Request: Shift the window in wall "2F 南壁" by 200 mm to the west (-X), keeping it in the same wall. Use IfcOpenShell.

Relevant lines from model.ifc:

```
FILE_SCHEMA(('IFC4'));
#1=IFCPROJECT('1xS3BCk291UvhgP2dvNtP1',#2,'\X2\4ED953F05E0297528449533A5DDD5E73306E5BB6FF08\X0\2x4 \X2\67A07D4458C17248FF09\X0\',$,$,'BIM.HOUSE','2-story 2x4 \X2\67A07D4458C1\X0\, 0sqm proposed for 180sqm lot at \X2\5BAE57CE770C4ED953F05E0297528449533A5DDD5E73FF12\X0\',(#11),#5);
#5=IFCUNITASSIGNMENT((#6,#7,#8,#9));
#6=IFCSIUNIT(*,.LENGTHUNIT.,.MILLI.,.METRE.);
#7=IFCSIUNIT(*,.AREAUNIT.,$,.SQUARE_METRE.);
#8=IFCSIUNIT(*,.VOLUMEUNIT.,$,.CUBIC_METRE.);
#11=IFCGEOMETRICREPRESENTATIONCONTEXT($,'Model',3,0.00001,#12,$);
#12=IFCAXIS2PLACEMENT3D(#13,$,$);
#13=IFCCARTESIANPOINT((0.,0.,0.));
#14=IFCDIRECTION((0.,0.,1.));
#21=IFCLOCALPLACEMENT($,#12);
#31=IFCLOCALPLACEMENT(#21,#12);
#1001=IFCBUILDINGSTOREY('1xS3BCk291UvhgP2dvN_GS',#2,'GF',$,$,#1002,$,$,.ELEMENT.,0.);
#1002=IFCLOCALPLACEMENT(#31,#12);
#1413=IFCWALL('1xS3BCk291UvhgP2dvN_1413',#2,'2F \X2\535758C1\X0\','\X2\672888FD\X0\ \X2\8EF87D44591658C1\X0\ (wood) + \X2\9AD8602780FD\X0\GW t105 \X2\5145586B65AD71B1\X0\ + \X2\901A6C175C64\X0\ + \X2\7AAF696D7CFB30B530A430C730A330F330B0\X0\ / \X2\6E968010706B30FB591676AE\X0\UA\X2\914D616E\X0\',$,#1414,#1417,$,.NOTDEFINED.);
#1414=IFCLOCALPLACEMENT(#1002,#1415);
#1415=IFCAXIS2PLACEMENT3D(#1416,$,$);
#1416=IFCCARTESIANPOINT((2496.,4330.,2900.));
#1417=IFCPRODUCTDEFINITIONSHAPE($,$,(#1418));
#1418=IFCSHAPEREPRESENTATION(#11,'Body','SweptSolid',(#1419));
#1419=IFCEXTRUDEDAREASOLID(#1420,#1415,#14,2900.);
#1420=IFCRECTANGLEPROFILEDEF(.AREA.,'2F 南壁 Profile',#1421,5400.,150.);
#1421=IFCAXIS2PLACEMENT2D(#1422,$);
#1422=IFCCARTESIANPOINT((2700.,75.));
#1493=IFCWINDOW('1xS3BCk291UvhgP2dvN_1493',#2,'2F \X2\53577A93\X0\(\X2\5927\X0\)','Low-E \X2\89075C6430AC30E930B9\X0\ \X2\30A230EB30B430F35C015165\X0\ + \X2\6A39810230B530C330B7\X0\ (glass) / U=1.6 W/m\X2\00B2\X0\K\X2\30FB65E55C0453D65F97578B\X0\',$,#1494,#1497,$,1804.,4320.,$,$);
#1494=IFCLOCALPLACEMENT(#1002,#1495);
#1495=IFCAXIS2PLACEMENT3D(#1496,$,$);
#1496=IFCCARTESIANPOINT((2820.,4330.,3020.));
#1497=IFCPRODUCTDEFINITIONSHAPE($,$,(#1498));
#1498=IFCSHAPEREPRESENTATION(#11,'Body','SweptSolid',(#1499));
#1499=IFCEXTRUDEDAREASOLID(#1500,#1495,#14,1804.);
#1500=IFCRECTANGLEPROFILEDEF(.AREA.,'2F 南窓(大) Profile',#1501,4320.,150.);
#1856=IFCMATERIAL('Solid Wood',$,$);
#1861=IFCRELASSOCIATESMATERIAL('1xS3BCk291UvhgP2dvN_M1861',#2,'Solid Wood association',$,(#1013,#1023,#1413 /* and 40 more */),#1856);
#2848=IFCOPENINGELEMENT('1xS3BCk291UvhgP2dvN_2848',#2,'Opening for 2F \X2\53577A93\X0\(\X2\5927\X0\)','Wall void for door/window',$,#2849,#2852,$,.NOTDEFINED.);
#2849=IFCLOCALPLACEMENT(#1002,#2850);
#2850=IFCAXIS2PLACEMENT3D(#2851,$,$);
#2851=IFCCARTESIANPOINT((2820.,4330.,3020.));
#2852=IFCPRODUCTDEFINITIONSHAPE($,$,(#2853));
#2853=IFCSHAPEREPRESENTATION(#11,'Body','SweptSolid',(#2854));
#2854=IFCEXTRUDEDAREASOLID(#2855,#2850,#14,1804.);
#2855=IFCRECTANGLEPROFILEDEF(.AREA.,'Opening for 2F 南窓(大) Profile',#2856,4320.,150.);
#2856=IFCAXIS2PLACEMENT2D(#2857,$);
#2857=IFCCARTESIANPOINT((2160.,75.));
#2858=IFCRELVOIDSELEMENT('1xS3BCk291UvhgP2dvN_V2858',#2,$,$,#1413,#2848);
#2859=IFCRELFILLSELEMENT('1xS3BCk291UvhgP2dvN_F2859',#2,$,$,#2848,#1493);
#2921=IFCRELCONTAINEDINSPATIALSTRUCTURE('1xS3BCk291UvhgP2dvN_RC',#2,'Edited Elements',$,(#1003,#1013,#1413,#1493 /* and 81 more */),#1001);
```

```python
import ifcopenshell
import ifcopenshell.api.geometry
import ifcopenshell.util.placement

model = ifcopenshell.open("model.ifc")

window = model.by_id(1493)
opening = window.FillsVoids[0].RelatingOpeningElement
wall = opening.VoidsElements[0].RelatingBuildingElement

wall_matrix = ifcopenshell.util.placement.get_local_placement(wall.ObjectPlacement)
shift = wall_matrix[:3, 0] * -200.0
before = ifcopenshell.util.placement.get_local_placement(window.ObjectPlacement)[:3, 3].copy()

# The window is not placed relative to its opening, so move both.
for product in (opening, window):
    matrix = ifcopenshell.util.placement.get_local_placement(product.ObjectPlacement)
    matrix[:3, 3] += shift
    ifcopenshell.api.geometry.edit_object_placement(model, product=product, matrix=matrix, is_si=False)

after = ifcopenshell.util.placement.get_local_placement(window.ObjectPlacement)[:3, 3]
print("window moved by", (after - before).round(3) + 0.0)

model.write("model_rev.ifc")
```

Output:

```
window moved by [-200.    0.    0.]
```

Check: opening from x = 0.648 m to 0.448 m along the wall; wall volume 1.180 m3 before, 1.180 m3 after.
